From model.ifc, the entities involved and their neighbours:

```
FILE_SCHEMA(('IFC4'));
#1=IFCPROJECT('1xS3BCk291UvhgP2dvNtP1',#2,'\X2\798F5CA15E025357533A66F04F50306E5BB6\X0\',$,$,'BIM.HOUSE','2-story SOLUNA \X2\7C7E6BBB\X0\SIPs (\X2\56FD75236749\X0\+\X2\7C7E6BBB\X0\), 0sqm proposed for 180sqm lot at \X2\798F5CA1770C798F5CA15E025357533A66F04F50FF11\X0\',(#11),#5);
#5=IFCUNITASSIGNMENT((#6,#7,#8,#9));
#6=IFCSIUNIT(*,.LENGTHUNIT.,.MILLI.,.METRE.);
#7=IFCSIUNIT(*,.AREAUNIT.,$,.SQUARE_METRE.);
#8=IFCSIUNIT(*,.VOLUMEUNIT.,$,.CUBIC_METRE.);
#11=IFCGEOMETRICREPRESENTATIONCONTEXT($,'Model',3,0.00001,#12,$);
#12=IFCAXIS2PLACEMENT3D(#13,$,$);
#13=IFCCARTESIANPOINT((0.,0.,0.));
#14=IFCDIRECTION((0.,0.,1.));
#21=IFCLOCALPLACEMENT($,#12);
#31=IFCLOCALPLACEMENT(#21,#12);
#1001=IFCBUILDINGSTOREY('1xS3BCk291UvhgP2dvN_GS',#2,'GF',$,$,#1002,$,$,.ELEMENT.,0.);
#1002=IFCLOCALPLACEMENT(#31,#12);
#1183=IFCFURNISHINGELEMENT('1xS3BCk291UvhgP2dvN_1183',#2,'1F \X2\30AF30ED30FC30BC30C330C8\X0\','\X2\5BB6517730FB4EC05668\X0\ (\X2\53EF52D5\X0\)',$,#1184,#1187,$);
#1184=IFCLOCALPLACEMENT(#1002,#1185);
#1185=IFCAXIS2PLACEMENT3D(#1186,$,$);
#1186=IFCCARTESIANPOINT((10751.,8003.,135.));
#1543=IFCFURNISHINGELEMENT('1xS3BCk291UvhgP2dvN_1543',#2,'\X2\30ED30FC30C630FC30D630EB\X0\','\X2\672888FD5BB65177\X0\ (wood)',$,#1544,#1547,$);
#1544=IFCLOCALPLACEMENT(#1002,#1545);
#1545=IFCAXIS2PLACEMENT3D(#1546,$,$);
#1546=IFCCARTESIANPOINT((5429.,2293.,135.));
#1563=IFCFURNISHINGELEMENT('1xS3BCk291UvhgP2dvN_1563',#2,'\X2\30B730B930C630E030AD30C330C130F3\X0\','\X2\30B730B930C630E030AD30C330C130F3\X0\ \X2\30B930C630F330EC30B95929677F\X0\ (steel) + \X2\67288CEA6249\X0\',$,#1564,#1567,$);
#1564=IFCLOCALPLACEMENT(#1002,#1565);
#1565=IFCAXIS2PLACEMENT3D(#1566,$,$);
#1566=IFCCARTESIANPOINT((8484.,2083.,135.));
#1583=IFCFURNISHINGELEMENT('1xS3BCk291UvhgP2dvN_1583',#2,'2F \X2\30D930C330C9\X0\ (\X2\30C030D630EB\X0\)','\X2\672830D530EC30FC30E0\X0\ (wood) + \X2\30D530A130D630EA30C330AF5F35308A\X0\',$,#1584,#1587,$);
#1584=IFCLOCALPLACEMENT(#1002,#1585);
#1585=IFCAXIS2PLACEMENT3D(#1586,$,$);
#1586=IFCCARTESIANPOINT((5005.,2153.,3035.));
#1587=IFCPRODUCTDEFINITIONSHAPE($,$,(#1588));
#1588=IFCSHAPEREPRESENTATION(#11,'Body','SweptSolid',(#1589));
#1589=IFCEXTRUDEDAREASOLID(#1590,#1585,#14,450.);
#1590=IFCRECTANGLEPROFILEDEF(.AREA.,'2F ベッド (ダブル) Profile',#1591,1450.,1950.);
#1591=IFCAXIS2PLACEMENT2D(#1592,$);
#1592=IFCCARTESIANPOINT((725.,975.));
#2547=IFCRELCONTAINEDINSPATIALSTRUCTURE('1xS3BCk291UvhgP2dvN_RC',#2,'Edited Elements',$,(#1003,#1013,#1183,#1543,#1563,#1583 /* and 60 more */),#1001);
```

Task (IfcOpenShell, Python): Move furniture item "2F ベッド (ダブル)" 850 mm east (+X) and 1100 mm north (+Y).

```python
import ifcopenshell
import ifcopenshell.api.geometry
import ifcopenshell.util.placement
import ifcopenshell.util.unit

model = ifcopenshell.open("model.ifc")
unit_scale = ifcopenshell.util.unit.calculate_unit_scale(model)

item = model.by_id(1583)
matrix = ifcopenshell.util.placement.get_local_placement(item.ObjectPlacement)
matrix[0, 3] += 0.85 / unit_scale
matrix[1, 3] += 1.1 / unit_scale
ifcopenshell.api.geometry.edit_object_placement(model, product=item, matrix=matrix, is_si=False)

print(ifcopenshell.util.placement.get_local_placement(item.ObjectPlacement).round(3) + 0.0)

model.write("model_v2.ifc")
```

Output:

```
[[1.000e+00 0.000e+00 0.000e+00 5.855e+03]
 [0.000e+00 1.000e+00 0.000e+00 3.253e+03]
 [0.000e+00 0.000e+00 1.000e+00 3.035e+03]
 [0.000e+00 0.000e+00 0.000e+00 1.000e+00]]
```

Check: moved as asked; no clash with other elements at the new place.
